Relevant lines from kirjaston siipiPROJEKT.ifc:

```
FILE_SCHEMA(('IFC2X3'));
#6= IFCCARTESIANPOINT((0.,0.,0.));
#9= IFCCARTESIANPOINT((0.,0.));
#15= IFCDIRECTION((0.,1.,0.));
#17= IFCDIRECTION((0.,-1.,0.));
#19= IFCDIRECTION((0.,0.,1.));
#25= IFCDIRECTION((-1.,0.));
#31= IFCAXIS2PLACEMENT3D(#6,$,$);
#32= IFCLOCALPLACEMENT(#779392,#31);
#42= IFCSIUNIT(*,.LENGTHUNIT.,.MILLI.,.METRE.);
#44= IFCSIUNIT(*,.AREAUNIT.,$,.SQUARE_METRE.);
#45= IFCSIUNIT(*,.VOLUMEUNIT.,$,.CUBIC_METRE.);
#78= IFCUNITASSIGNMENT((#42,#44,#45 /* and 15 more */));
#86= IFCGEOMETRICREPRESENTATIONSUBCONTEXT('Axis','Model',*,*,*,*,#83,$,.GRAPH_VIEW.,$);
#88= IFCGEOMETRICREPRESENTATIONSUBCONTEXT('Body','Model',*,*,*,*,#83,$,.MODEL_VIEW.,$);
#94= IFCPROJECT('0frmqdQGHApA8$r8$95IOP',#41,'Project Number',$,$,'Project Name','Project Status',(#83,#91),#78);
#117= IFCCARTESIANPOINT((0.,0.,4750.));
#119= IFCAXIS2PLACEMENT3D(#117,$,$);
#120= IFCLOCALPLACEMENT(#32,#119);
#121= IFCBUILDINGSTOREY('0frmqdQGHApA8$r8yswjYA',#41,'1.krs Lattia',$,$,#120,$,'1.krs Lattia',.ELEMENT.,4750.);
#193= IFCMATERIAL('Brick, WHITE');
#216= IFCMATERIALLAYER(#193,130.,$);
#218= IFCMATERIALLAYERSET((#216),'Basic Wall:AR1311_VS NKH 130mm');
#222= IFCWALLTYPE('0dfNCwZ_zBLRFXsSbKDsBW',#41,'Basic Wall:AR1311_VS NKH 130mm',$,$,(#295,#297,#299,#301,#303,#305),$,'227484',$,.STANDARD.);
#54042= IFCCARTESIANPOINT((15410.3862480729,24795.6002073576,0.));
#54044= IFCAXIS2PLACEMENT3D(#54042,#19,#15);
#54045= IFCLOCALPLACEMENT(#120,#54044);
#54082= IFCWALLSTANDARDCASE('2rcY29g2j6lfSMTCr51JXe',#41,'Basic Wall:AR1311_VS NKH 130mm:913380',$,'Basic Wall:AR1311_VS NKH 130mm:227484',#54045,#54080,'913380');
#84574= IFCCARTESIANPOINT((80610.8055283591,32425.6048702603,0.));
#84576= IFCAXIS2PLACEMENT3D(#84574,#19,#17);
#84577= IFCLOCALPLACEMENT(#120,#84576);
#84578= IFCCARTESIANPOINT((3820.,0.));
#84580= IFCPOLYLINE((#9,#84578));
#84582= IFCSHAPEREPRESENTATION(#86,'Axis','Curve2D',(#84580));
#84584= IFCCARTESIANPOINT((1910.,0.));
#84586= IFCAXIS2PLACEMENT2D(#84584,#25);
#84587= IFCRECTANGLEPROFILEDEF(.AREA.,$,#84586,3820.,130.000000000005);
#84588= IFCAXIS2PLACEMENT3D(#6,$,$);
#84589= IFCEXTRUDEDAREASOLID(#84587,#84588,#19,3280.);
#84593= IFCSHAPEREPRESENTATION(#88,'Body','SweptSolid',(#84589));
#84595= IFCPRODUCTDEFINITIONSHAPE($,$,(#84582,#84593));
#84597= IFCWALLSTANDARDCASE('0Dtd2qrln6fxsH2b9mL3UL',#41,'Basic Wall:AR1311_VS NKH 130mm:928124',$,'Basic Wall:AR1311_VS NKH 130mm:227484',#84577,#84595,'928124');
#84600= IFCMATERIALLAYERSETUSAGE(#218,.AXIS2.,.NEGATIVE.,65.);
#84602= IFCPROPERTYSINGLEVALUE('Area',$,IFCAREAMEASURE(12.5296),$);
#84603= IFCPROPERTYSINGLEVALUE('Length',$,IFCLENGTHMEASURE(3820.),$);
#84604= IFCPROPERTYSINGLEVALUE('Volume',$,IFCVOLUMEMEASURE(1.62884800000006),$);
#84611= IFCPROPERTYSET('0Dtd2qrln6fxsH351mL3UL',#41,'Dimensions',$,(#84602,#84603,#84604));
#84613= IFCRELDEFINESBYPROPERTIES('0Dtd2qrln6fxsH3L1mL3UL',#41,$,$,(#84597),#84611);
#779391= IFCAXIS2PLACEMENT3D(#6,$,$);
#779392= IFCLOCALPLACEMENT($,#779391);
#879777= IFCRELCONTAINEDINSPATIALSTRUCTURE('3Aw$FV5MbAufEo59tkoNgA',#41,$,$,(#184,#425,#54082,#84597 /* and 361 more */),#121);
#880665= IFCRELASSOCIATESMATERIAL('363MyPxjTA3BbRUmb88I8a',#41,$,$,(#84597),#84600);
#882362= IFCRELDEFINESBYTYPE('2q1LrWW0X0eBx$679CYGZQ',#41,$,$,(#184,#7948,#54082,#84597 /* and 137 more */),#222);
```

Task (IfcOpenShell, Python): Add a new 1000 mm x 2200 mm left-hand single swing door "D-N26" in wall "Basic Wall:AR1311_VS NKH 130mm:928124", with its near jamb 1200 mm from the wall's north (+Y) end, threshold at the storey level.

```python
import numpy as np
import ifcopenshell
import ifcopenshell.api.feature
import ifcopenshell.api.geometry
import ifcopenshell.api.pset
import ifcopenshell.api.root
import ifcopenshell.api.spatial
import ifcopenshell.api.type
import ifcopenshell.geom
import ifcopenshell.util.element
import ifcopenshell.util.placement
import ifcopenshell.util.representation
import ifcopenshell.util.shape
import ifcopenshell.util.unit

model = ifcopenshell.open("kirjaston siipiPROJEKT.ifc")
unit_scale = ifcopenshell.util.unit.calculate_unit_scale(model)
area_scale = ifcopenshell.util.unit.calculate_unit_scale(model, "AREAUNIT")
volume_scale = ifcopenshell.util.unit.calculate_unit_scale(model, "VOLUMEUNIT")
settings = ifcopenshell.geom.settings()


def volume(element):
    """Net volume in cubic metres, openings subtracted."""
    shape = ifcopenshell.geom.create_shape(settings, element)
    return ifcopenshell.util.shape.get_volume(shape.geometry)


wall = model.by_guid("0Dtd2qrln6fxsH2b9mL3UL")
storey = ifcopenshell.util.element.get_container(wall, ifc_class="IfcBuildingStorey")
context = ifcopenshell.util.representation.get_context(model, "Model", "Body", "MODEL_VIEW")
before = volume(wall)

width, height, from_end, sill = 1, 2.2, 1.2, 0.0  # metres

# The wall runs along its own X axis, and the end named is its -X end.
wall_shape = ifcopenshell.geom.create_shape(settings, wall)
x, y, z = ifcopenshell.util.shape.get_vertices(wall_shape.geometry).T
start = x.min() + from_end
face, thickness = float(y.min()), float(y.max() - y.min())
wall_matrix = ifcopenshell.util.placement.get_local_placement(wall.ObjectPlacement)
level = ifcopenshell.util.placement.get_local_placement(storey.ObjectPlacement)[2, 3]


def in_wall(x, y):
    """Placement at x, y metres in the wall's axes, at sill height."""
    matrix = wall_matrix.copy()
    matrix[:, 3] = wall_matrix @ np.array([x / unit_scale, y / unit_scale, 0.0, 1.0])
    matrix[2, 3] = level + sill / unit_scale
    return matrix


# Opening: a box that overshoots both wall faces by 50 mm.
opening = ifcopenshell.api.root.create_entity(model, ifc_class="IfcOpeningElement")
box = ifcopenshell.api.geometry.add_wall_representation(
    model, context=context, length=width, height=height, thickness=thickness + 0.1
)
ifcopenshell.api.geometry.assign_representation(model, product=opening, representation=box)
ifcopenshell.api.geometry.edit_object_placement(model, product=opening, matrix=in_wall(start, face - 0.05), is_si=False)
ifcopenshell.api.feature.add_feature(model, feature=opening, element=wall)

door = ifcopenshell.api.root.create_entity(model, ifc_class="IfcDoor", name="D-N26")
door.OverallWidth, door.OverallHeight = width / unit_scale, height / unit_scale
body = ifcopenshell.api.geometry.add_door_representation(
    model,
    context=context,
    overall_width=door.OverallWidth,
    overall_height=door.OverallHeight,
    operation_type="SINGLE_SWING_LEFT",
    lining_properties={"LiningDepth": thickness / unit_scale, "ThresholdDepth": thickness / unit_scale},
)
ifcopenshell.api.geometry.assign_representation(model, product=door, representation=body)
ifcopenshell.api.spatial.assign_container(model, products=[door], relating_structure=storey)
fills = ifcopenshell.api.feature.add_filling(model, opening=opening, element=door)
fills.OwnerHistory = door.OwnerHistory  # required in IFC2X3

# IFC2X3 keeps the operation on the door style.
style = ifcopenshell.api.root.create_entity(model, ifc_class="IfcDoorStyle", name="D-N26")
style.OperationType, style.ConstructionType = "SINGLE_SWING_LEFT", "NOTDEFINED"
style.ParameterTakesPrecedence = style.Sizeable = False
ifcopenshell.api.type.assign_type(model, related_objects=[door], relating_type=style)

# The lining spans the wall, so the door starts at the wall face.
ifcopenshell.api.geometry.edit_object_placement(model, product=door, matrix=in_wall(start, face), is_si=False)

after = volume(wall)

# Update the wall's stored quantities.
pset = model.by_id(ifcopenshell.util.element.get_pset(wall, "Dimensions", should_inherit=False)["id"])
ifcopenshell.api.pset.edit_pset(model, pset=pset, properties={
    "Area": model.create_entity("IfcAreaMeasure", after / thickness / area_scale),
    "Volume": model.create_entity("IfcVolumeMeasure", after / volume_scale),
})

print(f"wall volume {before:.3f} -> {after:.3f} m3")

model.write("kirjaston siipiPROJEKT-out.ifc")
```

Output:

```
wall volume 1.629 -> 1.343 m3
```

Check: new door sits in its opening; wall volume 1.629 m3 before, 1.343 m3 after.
